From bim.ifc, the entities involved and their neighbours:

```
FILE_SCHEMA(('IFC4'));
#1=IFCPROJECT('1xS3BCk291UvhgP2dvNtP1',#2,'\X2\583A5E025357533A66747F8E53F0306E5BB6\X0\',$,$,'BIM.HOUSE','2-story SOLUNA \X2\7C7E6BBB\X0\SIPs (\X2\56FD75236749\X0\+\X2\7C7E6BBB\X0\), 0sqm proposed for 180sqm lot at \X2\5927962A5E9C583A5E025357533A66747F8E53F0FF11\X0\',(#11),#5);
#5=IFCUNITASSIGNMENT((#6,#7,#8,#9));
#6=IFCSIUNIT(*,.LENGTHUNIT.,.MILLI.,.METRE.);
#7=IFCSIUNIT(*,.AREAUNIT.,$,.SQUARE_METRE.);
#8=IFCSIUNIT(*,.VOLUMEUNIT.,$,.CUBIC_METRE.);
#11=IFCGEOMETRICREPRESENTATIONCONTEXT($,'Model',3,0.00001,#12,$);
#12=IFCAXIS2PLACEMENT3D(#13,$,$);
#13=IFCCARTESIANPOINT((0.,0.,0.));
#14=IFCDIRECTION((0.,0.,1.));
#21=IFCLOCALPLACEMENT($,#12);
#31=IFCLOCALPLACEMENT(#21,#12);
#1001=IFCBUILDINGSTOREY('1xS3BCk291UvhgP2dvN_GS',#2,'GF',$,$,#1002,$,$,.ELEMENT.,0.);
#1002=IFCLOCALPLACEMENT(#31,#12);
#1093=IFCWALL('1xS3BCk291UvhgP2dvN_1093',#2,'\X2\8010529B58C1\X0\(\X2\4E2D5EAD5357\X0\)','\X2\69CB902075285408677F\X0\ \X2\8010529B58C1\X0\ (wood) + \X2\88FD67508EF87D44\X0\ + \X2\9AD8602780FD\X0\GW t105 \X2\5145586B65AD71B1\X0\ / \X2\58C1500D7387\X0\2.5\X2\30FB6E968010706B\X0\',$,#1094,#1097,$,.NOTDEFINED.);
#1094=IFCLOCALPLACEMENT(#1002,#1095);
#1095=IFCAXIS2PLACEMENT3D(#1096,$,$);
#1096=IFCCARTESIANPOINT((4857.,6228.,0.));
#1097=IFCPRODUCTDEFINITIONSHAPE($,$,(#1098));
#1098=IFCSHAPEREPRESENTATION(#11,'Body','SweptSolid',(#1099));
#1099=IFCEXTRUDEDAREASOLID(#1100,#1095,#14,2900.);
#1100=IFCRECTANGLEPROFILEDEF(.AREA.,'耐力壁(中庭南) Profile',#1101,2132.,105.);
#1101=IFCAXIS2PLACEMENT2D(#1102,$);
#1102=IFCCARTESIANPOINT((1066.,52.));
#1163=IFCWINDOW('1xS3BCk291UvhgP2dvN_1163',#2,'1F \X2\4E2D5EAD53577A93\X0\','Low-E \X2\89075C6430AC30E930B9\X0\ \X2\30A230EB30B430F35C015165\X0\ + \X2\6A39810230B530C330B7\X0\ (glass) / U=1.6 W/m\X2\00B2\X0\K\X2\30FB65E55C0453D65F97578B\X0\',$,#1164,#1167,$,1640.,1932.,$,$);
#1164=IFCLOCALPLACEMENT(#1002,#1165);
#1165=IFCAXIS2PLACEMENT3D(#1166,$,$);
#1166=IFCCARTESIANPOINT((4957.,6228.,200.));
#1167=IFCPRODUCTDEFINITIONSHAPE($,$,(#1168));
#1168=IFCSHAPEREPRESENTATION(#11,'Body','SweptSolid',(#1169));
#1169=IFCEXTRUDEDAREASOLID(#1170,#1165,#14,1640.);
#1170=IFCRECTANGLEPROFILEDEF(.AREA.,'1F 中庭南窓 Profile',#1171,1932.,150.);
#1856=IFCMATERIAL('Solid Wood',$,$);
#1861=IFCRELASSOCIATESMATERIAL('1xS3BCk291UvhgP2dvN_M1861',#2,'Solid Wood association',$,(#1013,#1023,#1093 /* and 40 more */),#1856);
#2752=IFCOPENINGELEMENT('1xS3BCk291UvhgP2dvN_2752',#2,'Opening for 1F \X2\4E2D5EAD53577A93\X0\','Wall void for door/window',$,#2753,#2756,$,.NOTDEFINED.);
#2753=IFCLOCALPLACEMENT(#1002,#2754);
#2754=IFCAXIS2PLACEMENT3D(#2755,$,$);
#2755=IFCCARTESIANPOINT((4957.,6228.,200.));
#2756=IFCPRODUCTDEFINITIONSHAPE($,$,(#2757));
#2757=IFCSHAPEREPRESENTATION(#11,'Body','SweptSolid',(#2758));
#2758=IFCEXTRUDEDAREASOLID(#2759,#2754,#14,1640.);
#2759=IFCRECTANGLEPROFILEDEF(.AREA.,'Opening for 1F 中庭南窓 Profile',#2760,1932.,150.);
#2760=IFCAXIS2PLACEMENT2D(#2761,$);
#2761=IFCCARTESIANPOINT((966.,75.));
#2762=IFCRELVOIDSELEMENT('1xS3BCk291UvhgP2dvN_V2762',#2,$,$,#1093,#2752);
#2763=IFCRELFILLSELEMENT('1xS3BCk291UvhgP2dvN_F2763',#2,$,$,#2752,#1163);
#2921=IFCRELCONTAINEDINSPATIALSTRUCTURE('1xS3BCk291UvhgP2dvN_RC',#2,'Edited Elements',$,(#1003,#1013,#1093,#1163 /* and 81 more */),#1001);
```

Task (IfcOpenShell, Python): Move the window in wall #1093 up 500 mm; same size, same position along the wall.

```python
import numpy as np
import ifcopenshell
import ifcopenshell.api.geometry
import ifcopenshell.util.placement
import ifcopenshell.util.unit

model = ifcopenshell.open("bim.ifc")
unit_scale = ifcopenshell.util.unit.calculate_unit_scale(model)

window = model.by_guid("1xS3BCk291UvhgP2dvN_1163")
opening = window.FillsVoids[0].RelatingOpeningElement
dz = 0.5 / unit_scale

shift = np.array([0.0, 0.0, dz])
# The window is not placed relative to its opening, so move both.
for product in (opening, window):
    matrix = ifcopenshell.util.placement.get_local_placement(product.ObjectPlacement)
    matrix[:3, 3] += shift
    ifcopenshell.api.geometry.edit_object_placement(model, product=product, matrix=matrix, is_si=False)

print(f"moved by {dz * unit_scale:+.3f} m")

model.write("bim_updated.ifc")
```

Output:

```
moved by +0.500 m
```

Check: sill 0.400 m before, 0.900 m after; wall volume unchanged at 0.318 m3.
